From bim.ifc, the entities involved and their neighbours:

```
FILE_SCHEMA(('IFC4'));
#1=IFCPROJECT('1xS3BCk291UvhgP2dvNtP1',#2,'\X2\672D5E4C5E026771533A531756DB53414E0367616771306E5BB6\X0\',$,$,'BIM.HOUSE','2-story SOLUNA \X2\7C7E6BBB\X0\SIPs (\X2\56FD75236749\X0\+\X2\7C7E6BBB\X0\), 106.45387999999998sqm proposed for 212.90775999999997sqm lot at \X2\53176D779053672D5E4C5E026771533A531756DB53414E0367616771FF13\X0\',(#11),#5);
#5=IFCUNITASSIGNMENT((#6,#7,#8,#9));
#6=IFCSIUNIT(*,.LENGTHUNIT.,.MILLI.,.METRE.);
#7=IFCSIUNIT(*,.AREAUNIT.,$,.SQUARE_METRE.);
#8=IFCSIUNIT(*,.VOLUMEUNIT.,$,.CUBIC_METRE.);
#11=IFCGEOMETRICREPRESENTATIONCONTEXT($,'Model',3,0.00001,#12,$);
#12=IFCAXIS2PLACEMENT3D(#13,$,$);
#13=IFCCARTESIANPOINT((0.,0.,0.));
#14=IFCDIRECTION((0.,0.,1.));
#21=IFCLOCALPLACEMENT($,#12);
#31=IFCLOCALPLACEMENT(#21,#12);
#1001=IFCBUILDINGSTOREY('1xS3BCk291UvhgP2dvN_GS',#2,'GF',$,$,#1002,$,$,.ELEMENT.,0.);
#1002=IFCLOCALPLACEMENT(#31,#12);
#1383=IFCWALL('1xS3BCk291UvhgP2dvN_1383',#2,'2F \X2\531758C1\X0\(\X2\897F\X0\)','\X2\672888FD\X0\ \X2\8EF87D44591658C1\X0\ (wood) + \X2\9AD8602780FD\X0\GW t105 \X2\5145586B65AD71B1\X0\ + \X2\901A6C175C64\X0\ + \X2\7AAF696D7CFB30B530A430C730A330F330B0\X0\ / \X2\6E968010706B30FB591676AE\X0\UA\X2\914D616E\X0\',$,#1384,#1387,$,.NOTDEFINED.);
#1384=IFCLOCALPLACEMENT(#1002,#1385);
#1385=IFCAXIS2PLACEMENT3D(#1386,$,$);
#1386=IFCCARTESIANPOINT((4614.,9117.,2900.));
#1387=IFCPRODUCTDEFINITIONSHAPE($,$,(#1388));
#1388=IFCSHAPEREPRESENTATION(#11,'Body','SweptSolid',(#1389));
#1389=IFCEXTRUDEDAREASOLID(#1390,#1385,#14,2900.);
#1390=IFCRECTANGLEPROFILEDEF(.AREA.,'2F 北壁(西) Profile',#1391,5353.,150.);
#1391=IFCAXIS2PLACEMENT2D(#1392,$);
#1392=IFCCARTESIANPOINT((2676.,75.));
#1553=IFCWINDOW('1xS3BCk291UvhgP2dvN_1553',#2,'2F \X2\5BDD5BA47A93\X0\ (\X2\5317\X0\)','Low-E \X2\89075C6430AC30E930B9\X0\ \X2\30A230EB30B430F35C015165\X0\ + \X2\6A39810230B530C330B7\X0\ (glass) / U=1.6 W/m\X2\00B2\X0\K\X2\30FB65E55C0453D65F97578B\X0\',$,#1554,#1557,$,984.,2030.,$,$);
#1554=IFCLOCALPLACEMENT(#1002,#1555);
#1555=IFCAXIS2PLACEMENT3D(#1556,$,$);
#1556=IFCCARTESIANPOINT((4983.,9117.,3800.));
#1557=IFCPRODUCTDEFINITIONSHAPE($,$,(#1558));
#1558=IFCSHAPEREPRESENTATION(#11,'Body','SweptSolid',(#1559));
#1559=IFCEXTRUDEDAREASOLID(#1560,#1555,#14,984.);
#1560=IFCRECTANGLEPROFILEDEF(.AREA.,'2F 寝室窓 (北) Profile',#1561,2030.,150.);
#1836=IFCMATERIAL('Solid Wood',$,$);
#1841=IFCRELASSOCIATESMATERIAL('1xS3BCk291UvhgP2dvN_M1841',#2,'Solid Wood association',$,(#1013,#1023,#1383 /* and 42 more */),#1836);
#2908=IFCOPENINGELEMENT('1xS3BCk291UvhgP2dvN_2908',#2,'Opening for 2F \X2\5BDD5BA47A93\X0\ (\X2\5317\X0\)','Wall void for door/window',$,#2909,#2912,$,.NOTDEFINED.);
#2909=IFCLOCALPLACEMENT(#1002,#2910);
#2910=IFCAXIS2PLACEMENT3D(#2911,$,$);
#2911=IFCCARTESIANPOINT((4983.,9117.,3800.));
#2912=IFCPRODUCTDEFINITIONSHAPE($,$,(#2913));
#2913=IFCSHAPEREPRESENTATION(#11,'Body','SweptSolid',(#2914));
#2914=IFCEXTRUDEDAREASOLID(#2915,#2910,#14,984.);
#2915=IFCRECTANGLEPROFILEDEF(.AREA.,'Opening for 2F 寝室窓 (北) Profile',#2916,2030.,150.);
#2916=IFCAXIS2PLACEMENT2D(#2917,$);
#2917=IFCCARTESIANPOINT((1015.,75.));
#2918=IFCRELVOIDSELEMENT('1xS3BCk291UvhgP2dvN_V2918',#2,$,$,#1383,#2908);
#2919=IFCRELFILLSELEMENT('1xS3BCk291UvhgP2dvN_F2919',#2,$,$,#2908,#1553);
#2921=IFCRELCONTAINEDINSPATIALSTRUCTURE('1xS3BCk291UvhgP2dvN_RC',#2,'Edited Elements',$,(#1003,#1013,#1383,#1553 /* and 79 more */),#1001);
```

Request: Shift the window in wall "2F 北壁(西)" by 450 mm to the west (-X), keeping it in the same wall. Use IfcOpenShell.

```python
import ifcopenshell
import ifcopenshell.api.geometry
import ifcopenshell.util.placement
import ifcopenshell.util.unit

model = ifcopenshell.open("bim.ifc")
unit_scale = ifcopenshell.util.unit.calculate_unit_scale(model)

window = model.by_guid("1xS3BCk291UvhgP2dvN_1553")
opening = window.FillsVoids[0].RelatingOpeningElement
wall = opening.VoidsElements[0].RelatingBuildingElement

wall_matrix = ifcopenshell.util.placement.get_local_placement(wall.ObjectPlacement)
shift = wall_matrix[:3, 0] * -0.45 / unit_scale
before = ifcopenshell.util.placement.get_local_placement(window.ObjectPlacement)[:3, 3].copy()

# The window is not placed relative to its opening, so move both.
for product in (opening, window):
    matrix = ifcopenshell.util.placement.get_local_placement(product.ObjectPlacement)
    matrix[:3, 3] += shift
    ifcopenshell.api.geometry.edit_object_placement(model, product=product, matrix=matrix, is_si=False)

after = ifcopenshell.util.placement.get_local_placement(window.ObjectPlacement)[:3, 3]
print("window moved by", (after - before).round(3) + 0.0)

model.write("bim_rev.ifc")
```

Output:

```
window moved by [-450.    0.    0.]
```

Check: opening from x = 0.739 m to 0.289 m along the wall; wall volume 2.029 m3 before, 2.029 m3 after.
